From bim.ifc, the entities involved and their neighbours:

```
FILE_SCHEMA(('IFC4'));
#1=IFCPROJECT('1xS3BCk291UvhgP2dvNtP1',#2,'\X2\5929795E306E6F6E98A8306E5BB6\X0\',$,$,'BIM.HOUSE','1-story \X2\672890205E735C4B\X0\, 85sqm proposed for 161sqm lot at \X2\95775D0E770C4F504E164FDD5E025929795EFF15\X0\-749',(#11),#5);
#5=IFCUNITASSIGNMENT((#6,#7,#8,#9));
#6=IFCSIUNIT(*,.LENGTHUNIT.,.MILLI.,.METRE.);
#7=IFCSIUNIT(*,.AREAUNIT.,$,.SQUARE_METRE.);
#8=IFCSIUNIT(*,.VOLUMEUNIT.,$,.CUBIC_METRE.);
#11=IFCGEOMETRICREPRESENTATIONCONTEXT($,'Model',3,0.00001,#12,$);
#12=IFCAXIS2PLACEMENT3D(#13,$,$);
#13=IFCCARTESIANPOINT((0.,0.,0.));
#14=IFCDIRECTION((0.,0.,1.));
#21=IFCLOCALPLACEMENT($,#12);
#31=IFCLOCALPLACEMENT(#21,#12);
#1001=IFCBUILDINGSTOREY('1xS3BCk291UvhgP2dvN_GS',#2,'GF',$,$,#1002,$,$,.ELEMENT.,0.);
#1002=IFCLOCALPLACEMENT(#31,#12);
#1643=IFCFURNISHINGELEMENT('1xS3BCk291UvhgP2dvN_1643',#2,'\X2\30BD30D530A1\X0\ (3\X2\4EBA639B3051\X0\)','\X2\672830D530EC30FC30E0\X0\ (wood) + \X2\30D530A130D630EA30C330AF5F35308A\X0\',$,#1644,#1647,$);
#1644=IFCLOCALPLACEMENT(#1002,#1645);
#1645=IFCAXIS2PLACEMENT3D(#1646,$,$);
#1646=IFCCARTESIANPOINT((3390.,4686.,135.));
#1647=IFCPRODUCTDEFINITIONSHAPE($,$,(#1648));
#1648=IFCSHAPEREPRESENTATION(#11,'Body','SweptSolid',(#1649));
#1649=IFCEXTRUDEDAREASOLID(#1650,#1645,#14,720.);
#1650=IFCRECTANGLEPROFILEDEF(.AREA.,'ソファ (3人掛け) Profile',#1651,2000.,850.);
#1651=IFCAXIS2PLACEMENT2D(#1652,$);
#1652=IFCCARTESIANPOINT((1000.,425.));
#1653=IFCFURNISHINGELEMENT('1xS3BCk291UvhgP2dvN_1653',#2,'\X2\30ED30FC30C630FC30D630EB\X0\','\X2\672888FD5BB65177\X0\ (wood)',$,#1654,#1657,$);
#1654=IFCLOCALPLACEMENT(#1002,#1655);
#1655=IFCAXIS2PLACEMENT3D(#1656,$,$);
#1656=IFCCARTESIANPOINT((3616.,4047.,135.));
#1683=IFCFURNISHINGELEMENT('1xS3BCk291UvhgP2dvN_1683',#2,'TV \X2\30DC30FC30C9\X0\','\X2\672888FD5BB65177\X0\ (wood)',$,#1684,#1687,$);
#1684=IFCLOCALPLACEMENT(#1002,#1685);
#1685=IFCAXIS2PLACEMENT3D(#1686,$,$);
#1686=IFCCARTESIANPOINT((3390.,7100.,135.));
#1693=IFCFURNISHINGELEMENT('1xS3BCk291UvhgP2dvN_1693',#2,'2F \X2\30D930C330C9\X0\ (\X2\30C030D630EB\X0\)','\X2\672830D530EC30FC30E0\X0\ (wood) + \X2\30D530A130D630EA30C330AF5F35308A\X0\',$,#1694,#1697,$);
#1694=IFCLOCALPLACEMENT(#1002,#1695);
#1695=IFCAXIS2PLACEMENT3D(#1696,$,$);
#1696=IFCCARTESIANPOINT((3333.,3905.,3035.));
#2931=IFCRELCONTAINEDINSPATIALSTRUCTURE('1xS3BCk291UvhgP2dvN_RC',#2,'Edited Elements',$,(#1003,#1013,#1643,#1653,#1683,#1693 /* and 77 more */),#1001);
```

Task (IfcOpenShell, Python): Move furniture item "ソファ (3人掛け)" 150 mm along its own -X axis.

```python
import ifcopenshell
import ifcopenshell.api.geometry
import ifcopenshell.util.placement
import ifcopenshell.util.unit

model = ifcopenshell.open("bim.ifc")
unit_scale = ifcopenshell.util.unit.calculate_unit_scale(model)

item = model.by_guid("1xS3BCk291UvhgP2dvN_1643")
matrix = ifcopenshell.util.placement.get_local_placement(item.ObjectPlacement)
matrix[:3, 3] -= matrix[:3, 0] * 0.15 / unit_scale
ifcopenshell.api.geometry.edit_object_placement(model, product=item, matrix=matrix, is_si=False)

print(ifcopenshell.util.placement.get_local_placement(item.ObjectPlacement).round(3) + 0.0)

model.write("bim_v2.ifc")
```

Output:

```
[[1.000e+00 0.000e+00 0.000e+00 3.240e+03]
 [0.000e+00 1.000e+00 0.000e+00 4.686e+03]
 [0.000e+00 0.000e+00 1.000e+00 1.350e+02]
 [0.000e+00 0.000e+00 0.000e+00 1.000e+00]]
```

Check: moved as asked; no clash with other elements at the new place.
